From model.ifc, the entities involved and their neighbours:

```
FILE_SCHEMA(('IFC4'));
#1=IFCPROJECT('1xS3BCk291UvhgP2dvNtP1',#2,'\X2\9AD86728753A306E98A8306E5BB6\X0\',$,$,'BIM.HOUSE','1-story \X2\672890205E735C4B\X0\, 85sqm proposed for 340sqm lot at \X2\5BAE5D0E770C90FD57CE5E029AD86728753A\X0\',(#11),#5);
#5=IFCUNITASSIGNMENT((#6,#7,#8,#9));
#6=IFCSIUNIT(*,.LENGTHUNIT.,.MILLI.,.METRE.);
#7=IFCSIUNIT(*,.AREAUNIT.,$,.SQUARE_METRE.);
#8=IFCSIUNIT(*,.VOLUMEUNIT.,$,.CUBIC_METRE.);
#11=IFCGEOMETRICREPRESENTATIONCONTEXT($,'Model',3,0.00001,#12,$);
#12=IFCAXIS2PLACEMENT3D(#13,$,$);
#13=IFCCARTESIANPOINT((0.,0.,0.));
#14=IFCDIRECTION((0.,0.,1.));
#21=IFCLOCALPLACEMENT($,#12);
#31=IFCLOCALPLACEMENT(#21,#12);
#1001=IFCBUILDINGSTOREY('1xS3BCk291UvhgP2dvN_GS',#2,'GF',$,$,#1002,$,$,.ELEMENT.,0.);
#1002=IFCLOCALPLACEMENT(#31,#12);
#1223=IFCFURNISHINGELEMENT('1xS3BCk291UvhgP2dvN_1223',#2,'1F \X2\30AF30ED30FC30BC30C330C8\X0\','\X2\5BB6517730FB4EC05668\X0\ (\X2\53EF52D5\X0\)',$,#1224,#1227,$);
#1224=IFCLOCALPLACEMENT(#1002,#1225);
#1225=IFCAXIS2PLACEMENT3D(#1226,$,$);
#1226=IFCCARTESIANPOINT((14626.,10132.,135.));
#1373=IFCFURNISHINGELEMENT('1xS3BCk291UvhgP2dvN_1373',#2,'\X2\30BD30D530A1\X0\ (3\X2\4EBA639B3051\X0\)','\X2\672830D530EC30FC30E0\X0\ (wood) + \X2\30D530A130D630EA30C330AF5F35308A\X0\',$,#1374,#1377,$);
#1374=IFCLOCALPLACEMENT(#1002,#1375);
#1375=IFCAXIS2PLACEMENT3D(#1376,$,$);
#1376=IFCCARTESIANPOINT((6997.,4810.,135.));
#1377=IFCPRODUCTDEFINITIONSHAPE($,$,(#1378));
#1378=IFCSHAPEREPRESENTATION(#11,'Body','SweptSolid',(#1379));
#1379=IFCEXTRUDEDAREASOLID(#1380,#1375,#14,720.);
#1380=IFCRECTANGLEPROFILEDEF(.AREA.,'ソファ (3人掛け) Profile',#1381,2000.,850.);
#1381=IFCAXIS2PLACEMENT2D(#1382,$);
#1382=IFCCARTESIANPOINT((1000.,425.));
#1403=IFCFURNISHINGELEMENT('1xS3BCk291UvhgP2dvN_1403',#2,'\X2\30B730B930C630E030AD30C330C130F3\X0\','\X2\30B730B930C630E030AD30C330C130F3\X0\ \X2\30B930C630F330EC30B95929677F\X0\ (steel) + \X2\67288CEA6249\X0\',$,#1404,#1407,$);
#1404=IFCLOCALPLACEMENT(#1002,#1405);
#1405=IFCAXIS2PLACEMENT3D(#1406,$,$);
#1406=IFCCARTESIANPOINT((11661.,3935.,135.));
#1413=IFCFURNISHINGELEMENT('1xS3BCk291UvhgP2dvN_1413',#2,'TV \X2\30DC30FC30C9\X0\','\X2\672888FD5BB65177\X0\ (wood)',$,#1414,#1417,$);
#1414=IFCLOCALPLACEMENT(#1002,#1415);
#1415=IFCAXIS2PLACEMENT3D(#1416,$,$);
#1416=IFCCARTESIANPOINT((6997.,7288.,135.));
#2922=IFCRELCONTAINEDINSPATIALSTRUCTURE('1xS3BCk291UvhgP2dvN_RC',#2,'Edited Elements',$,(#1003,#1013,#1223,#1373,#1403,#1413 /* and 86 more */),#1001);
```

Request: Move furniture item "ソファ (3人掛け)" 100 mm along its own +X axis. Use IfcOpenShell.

```python
import ifcopenshell
import ifcopenshell.api.geometry
import ifcopenshell.util.placement
import ifcopenshell.util.unit

model = ifcopenshell.open("model.ifc")
unit_scale = ifcopenshell.util.unit.calculate_unit_scale(model)

item = model.by_id(1373)
matrix = ifcopenshell.util.placement.get_local_placement(item.ObjectPlacement)
matrix[:3, 3] += matrix[:3, 0] * 0.1 / unit_scale
ifcopenshell.api.geometry.edit_object_placement(model, product=item, matrix=matrix, is_si=False)

print(ifcopenshell.util.placement.get_local_placement(item.ObjectPlacement).round(3) + 0.0)

model.write("model_updated.ifc")
```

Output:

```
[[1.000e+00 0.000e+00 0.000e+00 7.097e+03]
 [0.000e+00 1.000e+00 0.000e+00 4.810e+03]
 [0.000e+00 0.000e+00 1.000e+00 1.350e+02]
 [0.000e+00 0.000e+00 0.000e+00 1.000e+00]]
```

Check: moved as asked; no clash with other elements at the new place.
